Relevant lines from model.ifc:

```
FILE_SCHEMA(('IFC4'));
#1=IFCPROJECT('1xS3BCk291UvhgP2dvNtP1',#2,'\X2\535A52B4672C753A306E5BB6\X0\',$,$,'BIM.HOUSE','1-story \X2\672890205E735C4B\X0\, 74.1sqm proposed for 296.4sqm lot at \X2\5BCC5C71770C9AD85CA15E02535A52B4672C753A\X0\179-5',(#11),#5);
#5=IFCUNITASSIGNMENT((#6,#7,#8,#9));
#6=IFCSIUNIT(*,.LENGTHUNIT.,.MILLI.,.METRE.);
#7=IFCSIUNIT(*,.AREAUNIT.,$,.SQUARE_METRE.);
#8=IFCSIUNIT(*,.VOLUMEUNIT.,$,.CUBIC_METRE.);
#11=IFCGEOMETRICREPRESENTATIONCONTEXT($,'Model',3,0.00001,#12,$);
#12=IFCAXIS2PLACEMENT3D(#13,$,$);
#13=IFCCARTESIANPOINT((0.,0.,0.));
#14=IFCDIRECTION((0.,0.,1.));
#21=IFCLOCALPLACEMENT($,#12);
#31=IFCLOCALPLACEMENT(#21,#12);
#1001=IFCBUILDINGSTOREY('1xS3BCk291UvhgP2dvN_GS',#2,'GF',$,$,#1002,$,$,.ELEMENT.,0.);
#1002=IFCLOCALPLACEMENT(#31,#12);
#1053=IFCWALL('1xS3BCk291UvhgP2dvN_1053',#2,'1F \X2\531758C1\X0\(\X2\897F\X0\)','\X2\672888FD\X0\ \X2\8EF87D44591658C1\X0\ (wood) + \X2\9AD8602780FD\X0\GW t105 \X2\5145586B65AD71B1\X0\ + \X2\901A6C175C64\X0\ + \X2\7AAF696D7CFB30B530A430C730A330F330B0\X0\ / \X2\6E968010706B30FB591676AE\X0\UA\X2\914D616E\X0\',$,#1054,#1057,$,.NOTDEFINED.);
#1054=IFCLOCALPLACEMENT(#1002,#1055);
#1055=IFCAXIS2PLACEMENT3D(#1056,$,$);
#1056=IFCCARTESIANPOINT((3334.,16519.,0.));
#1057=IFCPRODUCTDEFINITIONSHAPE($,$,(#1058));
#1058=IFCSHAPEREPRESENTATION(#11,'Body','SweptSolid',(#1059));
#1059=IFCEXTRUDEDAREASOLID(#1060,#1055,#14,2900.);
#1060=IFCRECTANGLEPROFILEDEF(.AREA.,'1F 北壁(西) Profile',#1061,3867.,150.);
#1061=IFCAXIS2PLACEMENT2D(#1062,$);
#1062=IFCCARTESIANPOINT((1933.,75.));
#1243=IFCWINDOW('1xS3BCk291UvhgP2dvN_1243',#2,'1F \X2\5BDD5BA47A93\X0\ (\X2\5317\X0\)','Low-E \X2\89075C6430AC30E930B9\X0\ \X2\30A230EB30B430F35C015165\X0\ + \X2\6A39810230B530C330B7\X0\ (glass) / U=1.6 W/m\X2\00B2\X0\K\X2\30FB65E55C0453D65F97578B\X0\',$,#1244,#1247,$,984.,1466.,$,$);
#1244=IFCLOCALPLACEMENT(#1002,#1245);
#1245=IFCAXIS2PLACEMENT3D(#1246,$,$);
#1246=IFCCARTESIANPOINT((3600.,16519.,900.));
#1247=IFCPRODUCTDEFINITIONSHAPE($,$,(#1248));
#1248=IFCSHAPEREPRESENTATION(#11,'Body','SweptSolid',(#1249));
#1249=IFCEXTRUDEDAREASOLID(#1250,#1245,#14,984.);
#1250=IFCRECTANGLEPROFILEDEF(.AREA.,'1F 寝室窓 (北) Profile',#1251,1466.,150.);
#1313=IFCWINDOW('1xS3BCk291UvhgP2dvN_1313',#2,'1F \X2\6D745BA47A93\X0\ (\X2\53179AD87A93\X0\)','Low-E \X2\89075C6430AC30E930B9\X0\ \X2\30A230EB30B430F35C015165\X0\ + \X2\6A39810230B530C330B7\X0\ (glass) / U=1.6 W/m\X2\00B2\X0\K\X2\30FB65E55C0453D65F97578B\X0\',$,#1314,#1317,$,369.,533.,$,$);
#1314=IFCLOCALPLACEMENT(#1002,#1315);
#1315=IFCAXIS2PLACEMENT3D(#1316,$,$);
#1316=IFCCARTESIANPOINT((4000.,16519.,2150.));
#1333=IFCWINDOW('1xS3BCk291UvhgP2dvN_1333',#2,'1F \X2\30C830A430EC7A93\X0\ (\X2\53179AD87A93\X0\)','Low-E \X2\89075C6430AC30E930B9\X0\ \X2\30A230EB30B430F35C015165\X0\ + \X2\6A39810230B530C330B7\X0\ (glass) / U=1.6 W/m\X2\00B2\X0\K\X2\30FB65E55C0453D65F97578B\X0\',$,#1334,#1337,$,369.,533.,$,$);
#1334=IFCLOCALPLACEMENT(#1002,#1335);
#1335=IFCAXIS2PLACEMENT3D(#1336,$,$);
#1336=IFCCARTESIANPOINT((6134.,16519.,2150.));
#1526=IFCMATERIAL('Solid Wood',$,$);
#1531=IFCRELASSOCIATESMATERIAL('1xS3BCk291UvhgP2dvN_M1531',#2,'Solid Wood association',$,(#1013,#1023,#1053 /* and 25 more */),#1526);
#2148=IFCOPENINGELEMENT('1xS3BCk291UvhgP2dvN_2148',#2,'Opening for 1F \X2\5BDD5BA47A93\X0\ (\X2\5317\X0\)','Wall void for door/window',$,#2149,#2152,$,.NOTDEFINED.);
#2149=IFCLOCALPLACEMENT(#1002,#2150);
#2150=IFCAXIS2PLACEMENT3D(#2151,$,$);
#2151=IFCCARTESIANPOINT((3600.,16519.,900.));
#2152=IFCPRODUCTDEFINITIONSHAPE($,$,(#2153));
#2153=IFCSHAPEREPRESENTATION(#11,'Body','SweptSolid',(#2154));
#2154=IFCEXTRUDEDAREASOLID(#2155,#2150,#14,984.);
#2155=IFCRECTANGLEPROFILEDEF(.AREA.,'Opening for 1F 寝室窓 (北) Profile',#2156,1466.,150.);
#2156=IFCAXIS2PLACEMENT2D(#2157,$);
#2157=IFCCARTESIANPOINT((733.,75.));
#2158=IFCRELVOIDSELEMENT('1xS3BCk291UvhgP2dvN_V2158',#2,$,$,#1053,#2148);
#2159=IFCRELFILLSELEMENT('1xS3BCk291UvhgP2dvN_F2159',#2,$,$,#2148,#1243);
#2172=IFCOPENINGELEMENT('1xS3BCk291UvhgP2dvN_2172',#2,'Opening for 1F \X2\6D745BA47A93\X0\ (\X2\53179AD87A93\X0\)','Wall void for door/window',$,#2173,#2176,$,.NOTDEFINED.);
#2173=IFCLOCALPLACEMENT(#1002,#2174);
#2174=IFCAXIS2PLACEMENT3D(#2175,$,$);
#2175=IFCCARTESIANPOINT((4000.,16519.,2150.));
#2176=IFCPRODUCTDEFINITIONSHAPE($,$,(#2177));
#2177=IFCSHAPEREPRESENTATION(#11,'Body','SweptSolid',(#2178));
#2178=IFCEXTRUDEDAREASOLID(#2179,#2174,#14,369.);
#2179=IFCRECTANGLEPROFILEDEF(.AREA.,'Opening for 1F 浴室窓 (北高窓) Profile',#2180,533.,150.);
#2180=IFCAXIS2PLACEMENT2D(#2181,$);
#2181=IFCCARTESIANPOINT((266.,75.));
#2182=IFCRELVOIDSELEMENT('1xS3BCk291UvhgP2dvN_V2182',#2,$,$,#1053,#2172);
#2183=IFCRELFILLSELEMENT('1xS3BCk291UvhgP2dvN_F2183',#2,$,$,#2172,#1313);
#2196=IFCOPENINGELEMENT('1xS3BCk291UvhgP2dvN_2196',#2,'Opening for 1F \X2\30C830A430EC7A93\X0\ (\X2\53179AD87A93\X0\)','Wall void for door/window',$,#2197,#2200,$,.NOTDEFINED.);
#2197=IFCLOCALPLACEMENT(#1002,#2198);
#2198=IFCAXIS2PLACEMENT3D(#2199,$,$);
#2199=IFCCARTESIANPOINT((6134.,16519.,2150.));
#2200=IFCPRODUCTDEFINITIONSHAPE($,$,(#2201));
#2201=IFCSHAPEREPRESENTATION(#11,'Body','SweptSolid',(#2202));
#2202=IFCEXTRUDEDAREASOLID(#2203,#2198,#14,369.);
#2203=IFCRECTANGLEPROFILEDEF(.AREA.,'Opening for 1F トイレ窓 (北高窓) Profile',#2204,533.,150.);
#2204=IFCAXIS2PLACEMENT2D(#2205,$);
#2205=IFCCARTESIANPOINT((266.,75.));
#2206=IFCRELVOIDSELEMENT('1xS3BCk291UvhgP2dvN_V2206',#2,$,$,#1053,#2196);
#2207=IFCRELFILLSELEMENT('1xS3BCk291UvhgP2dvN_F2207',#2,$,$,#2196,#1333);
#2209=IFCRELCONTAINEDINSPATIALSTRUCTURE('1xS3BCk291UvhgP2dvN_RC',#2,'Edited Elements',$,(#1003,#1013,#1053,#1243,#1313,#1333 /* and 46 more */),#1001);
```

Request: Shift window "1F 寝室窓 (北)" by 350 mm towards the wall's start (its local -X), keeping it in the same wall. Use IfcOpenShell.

```python
import ifcopenshell
import ifcopenshell.api.geometry
import ifcopenshell.util.placement
import ifcopenshell.util.unit

model = ifcopenshell.open("model.ifc")
unit_scale = ifcopenshell.util.unit.calculate_unit_scale(model)

window = model.by_id(1243)
opening = window.FillsVoids[0].RelatingOpeningElement
wall = opening.VoidsElements[0].RelatingBuildingElement

wall_matrix = ifcopenshell.util.placement.get_local_placement(wall.ObjectPlacement)
shift = wall_matrix[:3, 0] * -0.35 / unit_scale
before = ifcopenshell.util.placement.get_local_placement(window.ObjectPlacement)[:3, 3].copy()

# The window is not placed relative to its opening, so move both.
for product in (opening, window):
    matrix = ifcopenshell.util.placement.get_local_placement(product.ObjectPlacement)
    matrix[:3, 3] += shift
    ifcopenshell.api.geometry.edit_object_placement(model, product=product, matrix=matrix, is_si=False)

after = ifcopenshell.util.placement.get_local_placement(window.ObjectPlacement)[:3, 3]
print("window moved by", (after - before).round(3) + 0.0)

model.write("model_updated.ifc")
```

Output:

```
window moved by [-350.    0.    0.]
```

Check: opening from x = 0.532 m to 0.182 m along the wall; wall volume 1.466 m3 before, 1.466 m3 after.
